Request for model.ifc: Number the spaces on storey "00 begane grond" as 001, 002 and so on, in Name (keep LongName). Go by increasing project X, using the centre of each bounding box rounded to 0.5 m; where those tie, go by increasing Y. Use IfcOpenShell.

First a look at what the model holds.

```python
import ifcopenshell
import ifcopenshell.util.element
import ifcopenshell.util.placement

model = ifcopenshell.open("model.ifc")
print(model.schema)
storey = next(s for s in model.by_type("IfcBuildingStorey") if s.Name == "00 begane grond")
spaces = [e for e in ifcopenshell.util.element.get_decomposition(storey) if e.is_a("IfcSpace")]
for e in sorted(spaces, key=lambda e: e.id()):
    origin = ifcopenshell.util.placement.get_local_placement(e.ObjectPlacement)[:3, 3]
    print(e.id(), e.Name, e.LongName, origin.round(2) + 0.0, sep=" | ")
```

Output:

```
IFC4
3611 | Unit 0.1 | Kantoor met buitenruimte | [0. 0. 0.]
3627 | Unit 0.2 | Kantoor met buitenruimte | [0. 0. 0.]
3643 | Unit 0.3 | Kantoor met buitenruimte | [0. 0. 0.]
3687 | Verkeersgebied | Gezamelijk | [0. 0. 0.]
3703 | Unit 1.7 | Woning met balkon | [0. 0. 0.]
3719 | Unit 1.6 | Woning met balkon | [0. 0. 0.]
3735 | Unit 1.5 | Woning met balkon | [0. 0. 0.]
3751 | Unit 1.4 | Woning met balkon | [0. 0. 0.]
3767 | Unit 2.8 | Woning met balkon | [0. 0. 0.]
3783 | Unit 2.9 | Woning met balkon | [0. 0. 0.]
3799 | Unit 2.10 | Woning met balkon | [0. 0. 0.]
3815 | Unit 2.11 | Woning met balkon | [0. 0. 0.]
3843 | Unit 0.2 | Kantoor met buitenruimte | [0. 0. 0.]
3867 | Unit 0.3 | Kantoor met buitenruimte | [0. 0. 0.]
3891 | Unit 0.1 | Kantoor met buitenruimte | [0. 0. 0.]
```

```python
import ifcopenshell
import ifcopenshell.geom
import ifcopenshell.util.element
import ifcopenshell.util.shape

model = ifcopenshell.open("model.ifc")
settings = ifcopenshell.geom.settings()
settings.set("use-world-coords", True)


def centre(element):
    shape = ifcopenshell.geom.create_shape(settings, element)
    return ifcopenshell.util.shape.get_bbox_centroid(shape.geometry)


storey = next(s for s in model.by_type("IfcBuildingStorey") if s.Name == "00 begane grond")
spaces = [e for e in ifcopenshell.util.element.get_decomposition(storey) if e.is_a("IfcSpace")]

# Insertion points can sit at a corner or the storey origin, so sort by the geometry (in metres).
centres = {e: centre(e) for e in spaces}
spaces.sort(key=lambda e: (round(centres[e][0] / 0.5), centres[e][1]))

for i, e in enumerate(spaces, start=1):
    number = f"0{i:02d}"
    e.Name = number
    print(e.id(), number)

model.write("model_updated.ifc")
```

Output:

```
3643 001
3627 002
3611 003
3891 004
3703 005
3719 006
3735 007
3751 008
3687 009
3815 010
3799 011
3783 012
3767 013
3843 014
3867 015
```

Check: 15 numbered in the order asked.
